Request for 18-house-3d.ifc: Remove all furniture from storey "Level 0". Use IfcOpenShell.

First a look at what the model holds.

```python
import ifcopenshell
import ifcopenshell.util.element

model = ifcopenshell.open("18-house-3d.ifc")
print(model.schema)
storey = next(s for s in model.by_type("IfcBuildingStorey") if s.Name == "Level 0")
furniture = [e for e in ifcopenshell.util.element.get_decomposition(storey) if e.is_a("IfcFurnishingElement")]
seen = {}
for e in furniture:
    element_type = ifcopenshell.util.element.get_type(e)
    name = element_type.Name if element_type not in (None, e) else None
    seen[name] = seen.get(name, 0) + 1
for name, count in sorted(seen.items(), key=str):
    print(count, "x", name)
```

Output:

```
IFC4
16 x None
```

```python
import ifcopenshell
import ifcopenshell.api.root
import ifcopenshell.util.element

model = ifcopenshell.open("18-house-3d.ifc")

storey = next(s for s in model.by_type("IfcBuildingStorey") if s.Name == "Level 0")
furniture = [e for e in ifcopenshell.util.element.get_decomposition(storey) if e.is_a("IfcFurnishingElement")]

for e in furniture:
    ifcopenshell.api.root.remove_product(model, product=e)
print(len(furniture), "removed")

model.write("18-house-3d_rev.ifc")
```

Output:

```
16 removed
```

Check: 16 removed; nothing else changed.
